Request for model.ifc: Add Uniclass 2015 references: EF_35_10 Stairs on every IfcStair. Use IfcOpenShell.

First a look at what the model holds.

```python
import ifcopenshell

model = ifcopenshell.open("model.ifc")
print(model.schema)
print("classifications:", [c.Name for c in model.by_type("IfcClassification")])
for ifc_class in ("IfcDoor", "IfcRoof", "IfcStair", "IfcWall", "IfcWindow"):
    print(ifc_class, len(model.by_type(ifc_class)))
```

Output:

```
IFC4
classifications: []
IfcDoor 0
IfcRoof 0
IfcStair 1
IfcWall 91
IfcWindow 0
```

```python
import ifcopenshell
import ifcopenshell.api.classification

model = ifcopenshell.open("model.ifc")

system = ifcopenshell.api.classification.add_classification(model, classification="Uniclass 2015")

codes = {
    "IfcStair": ("EF_35_10", "Stairs"),
}
for ifc_class, (code, name) in codes.items():
    products = model.by_type(ifc_class)
    ifcopenshell.api.classification.add_reference(
        model, products=products, classification=system, identification=code, name=name
    )
    print(code, len(products))

model.write("model-out.ifc")
```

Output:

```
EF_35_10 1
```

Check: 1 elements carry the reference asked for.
